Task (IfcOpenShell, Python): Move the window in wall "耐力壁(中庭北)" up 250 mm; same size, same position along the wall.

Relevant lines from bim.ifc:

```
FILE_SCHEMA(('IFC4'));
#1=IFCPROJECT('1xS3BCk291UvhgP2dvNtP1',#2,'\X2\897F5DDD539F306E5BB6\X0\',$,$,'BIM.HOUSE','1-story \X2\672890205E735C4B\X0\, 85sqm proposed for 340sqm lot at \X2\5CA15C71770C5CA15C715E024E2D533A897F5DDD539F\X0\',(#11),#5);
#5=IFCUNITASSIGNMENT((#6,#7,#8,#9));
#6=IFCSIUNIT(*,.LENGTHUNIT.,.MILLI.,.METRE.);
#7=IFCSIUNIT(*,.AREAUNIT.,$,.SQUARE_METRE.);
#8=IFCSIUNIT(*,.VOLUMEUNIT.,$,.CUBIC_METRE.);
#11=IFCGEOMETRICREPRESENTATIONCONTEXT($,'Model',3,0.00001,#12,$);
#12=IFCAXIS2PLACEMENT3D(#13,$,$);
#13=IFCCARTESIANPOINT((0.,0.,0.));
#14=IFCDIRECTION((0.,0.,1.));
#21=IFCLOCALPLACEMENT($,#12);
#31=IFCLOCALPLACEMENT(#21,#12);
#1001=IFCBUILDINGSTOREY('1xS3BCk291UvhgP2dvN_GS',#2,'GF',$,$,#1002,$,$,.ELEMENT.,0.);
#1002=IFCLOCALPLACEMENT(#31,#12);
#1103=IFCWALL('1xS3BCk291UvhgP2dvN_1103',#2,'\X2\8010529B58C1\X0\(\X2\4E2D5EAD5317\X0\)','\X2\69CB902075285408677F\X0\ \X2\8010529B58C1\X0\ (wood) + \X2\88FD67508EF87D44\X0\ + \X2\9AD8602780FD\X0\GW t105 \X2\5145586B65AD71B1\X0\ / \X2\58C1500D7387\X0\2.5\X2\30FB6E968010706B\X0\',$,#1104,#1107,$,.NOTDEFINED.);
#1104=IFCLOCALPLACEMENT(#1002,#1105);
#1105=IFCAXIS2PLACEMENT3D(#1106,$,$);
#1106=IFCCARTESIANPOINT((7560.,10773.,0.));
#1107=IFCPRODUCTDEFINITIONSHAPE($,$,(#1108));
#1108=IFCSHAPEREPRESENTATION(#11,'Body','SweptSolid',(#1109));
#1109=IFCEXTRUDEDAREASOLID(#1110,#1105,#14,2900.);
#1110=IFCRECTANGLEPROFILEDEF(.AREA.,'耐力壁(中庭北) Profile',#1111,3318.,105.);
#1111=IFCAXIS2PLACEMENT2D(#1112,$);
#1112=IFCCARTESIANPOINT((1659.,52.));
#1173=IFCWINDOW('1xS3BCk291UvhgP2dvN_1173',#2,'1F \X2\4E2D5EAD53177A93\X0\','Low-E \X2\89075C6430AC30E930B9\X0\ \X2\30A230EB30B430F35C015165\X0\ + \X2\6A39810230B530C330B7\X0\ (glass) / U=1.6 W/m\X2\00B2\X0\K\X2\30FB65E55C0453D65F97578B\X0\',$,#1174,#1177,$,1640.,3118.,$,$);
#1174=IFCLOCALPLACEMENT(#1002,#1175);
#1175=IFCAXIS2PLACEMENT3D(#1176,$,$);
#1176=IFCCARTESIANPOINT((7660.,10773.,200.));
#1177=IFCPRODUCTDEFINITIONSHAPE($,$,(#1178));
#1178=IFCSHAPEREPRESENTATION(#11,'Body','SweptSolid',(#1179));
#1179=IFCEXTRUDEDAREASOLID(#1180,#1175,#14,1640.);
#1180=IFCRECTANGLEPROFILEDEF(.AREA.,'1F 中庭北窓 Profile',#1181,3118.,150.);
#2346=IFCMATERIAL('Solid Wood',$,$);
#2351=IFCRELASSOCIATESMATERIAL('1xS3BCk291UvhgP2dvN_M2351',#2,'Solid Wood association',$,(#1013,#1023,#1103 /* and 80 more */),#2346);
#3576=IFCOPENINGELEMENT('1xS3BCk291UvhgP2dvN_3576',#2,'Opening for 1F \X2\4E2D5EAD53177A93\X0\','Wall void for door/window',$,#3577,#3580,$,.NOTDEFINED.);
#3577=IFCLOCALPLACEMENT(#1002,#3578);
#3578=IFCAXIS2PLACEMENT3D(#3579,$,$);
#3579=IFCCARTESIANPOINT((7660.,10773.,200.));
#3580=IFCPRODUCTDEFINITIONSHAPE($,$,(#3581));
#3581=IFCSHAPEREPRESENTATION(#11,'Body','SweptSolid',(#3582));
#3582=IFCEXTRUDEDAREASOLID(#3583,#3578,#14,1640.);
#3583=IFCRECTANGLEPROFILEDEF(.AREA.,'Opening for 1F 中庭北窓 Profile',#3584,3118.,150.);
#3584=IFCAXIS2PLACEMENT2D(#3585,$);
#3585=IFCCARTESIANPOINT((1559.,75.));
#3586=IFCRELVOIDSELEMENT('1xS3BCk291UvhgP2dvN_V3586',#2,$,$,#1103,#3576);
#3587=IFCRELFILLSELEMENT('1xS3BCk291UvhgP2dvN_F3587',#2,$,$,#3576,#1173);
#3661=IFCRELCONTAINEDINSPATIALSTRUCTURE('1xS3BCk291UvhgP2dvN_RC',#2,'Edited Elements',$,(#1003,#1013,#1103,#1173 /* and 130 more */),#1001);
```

```python
import numpy as np
import ifcopenshell
import ifcopenshell.api.geometry
import ifcopenshell.util.placement
import ifcopenshell.util.unit

model = ifcopenshell.open("bim.ifc")
unit_scale = ifcopenshell.util.unit.calculate_unit_scale(model)

window = model.by_guid("1xS3BCk291UvhgP2dvN_1173")
opening = window.FillsVoids[0].RelatingOpeningElement
dz = 0.25 / unit_scale

shift = np.array([0.0, 0.0, dz])
# The window is not placed relative to its opening, so move both.
for product in (opening, window):
    matrix = ifcopenshell.util.placement.get_local_placement(product.ObjectPlacement)
    matrix[:3, 3] += shift
    ifcopenshell.api.geometry.edit_object_placement(model, product=product, matrix=matrix, is_si=False)

print(f"moved by {dz * unit_scale:+.3f} m")

model.write("bim-out.ifc")
```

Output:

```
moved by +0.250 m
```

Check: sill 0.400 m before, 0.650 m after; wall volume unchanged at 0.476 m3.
